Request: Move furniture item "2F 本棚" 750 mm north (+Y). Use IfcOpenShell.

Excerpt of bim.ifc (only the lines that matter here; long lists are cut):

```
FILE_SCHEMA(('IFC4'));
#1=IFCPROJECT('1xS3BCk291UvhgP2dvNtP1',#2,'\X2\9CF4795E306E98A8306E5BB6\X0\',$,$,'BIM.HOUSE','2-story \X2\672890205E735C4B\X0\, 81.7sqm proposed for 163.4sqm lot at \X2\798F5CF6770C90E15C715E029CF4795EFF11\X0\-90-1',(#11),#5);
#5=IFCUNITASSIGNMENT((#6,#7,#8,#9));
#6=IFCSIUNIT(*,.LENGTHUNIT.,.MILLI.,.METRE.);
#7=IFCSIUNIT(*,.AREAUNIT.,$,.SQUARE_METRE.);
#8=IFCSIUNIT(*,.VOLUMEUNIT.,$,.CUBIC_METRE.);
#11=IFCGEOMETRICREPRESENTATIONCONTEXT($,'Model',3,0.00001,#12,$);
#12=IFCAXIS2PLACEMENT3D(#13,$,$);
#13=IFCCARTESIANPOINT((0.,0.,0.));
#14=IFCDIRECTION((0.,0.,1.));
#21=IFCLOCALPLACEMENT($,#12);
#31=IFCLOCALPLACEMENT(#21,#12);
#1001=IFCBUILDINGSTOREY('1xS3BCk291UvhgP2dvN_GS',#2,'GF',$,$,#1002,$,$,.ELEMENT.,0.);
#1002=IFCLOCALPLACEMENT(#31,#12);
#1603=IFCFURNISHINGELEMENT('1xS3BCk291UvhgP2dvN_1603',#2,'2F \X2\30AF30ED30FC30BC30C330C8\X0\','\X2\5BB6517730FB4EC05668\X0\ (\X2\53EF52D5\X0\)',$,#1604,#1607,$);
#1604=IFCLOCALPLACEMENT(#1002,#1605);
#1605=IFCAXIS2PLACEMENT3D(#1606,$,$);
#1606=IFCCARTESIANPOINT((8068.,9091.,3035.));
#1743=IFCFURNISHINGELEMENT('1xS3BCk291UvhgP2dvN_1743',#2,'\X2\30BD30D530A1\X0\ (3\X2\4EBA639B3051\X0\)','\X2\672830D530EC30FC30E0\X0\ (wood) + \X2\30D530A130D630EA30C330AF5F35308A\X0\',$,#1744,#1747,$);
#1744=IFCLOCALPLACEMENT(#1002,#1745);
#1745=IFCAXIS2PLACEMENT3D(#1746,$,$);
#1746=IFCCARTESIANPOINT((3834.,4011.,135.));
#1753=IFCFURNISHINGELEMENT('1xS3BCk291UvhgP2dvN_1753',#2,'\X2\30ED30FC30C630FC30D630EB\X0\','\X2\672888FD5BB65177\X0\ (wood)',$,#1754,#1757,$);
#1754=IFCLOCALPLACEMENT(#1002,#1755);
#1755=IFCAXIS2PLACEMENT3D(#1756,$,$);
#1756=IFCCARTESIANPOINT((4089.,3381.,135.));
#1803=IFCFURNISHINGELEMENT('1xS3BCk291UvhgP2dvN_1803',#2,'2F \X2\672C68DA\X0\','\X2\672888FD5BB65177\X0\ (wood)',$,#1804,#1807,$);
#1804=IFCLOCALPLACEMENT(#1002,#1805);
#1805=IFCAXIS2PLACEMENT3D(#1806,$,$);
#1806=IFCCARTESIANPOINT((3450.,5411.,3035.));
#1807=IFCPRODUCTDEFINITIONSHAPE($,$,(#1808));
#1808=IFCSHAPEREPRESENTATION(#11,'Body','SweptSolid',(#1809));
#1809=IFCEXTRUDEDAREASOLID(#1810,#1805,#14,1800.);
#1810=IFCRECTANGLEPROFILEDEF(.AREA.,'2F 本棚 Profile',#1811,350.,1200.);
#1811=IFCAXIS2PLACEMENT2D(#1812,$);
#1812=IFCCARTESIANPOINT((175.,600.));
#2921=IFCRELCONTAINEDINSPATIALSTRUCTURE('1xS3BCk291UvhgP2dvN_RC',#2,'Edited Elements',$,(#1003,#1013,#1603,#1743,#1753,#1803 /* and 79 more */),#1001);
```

```python
import ifcopenshell
import ifcopenshell.api.geometry
import ifcopenshell.util.placement
import ifcopenshell.util.unit

model = ifcopenshell.open("bim.ifc")
unit_scale = ifcopenshell.util.unit.calculate_unit_scale(model)

item = model.by_guid("1xS3BCk291UvhgP2dvN_1803")
matrix = ifcopenshell.util.placement.get_local_placement(item.ObjectPlacement)
matrix[1, 3] += 0.75 / unit_scale
ifcopenshell.api.geometry.edit_object_placement(model, product=item, matrix=matrix, is_si=False)

print(ifcopenshell.util.placement.get_local_placement(item.ObjectPlacement).round(3) + 0.0)

model.write("bim_updated.ifc")
```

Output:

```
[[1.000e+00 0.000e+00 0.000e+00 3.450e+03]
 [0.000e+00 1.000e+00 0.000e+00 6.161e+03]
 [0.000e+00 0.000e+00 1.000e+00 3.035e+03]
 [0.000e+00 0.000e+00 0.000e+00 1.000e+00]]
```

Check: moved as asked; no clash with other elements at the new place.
